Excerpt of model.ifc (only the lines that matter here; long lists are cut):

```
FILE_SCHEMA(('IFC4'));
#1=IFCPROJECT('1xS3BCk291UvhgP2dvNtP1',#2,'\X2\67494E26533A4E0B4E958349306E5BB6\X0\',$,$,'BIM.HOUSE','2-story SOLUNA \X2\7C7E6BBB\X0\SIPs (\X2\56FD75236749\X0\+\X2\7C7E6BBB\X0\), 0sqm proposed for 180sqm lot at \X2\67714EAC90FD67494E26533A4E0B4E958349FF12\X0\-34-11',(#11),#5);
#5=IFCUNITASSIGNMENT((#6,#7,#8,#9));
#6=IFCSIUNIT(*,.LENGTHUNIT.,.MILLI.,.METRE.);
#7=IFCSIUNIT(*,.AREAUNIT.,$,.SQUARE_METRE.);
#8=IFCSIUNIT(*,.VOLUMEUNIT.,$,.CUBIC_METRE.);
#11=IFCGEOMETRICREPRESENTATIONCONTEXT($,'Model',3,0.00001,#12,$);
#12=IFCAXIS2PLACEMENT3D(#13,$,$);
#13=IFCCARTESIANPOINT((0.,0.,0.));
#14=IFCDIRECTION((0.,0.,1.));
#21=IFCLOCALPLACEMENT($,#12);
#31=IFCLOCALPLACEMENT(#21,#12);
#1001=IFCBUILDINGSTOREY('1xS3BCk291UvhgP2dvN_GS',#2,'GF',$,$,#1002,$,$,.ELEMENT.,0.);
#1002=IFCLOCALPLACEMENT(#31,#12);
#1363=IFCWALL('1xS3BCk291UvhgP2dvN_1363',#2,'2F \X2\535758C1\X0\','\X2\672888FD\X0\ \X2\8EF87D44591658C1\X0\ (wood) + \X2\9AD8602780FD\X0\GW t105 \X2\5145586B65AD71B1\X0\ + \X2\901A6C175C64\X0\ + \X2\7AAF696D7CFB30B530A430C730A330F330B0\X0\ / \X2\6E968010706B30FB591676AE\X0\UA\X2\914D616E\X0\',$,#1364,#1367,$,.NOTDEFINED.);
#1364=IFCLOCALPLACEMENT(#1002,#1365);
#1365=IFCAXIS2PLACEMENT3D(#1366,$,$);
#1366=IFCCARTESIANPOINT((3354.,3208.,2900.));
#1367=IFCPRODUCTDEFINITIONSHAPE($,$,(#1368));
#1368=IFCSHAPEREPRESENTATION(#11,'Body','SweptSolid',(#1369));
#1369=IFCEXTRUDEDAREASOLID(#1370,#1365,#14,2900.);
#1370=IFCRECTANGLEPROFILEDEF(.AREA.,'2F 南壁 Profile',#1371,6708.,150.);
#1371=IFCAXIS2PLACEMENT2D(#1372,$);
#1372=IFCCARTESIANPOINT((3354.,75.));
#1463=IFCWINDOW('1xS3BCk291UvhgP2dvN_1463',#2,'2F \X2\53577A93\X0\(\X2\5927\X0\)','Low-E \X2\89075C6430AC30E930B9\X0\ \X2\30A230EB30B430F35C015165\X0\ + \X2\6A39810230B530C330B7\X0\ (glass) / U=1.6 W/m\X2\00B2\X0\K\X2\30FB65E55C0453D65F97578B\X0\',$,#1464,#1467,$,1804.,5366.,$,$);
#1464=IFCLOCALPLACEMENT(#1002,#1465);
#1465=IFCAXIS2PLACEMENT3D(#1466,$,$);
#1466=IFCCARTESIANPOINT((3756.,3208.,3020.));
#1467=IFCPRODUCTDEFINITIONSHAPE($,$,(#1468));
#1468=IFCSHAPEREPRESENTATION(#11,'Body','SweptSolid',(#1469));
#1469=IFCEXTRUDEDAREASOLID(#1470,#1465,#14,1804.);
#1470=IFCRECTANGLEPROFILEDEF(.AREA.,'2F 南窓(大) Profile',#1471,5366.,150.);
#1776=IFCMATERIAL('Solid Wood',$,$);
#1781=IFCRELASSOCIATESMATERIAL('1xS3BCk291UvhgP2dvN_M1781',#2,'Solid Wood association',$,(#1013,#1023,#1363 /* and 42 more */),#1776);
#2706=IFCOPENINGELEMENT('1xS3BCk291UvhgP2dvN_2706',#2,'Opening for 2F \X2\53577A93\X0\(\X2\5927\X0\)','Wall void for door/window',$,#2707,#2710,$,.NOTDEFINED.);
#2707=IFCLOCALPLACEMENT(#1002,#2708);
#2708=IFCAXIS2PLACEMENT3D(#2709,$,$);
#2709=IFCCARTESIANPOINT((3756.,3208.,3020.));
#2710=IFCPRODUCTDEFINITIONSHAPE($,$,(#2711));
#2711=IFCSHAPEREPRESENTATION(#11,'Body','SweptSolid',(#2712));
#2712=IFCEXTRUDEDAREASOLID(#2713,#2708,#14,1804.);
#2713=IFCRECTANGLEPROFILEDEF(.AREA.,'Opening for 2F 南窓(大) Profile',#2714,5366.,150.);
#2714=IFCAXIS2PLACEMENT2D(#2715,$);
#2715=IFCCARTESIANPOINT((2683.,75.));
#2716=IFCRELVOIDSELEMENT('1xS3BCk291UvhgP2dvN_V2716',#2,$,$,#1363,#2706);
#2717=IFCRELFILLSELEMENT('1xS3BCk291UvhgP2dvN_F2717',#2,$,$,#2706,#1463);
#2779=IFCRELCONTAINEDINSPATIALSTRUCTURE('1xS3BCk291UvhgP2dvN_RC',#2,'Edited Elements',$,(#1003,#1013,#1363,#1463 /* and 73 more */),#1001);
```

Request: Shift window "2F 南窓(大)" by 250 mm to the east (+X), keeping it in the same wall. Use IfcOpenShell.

```python
import ifcopenshell
import ifcopenshell.api.geometry
import ifcopenshell.util.placement
import ifcopenshell.util.unit

model = ifcopenshell.open("model.ifc")
unit_scale = ifcopenshell.util.unit.calculate_unit_scale(model)

window = model.by_guid("1xS3BCk291UvhgP2dvN_1463")
opening = window.FillsVoids[0].RelatingOpeningElement
wall = opening.VoidsElements[0].RelatingBuildingElement

wall_matrix = ifcopenshell.util.placement.get_local_placement(wall.ObjectPlacement)
shift = wall_matrix[:3, 0] * 0.25 / unit_scale
before = ifcopenshell.util.placement.get_local_placement(window.ObjectPlacement)[:3, 3].copy()

# The window is not placed relative to its opening, so move both.
for product in (opening, window):
    matrix = ifcopenshell.util.placement.get_local_placement(product.ObjectPlacement)
    matrix[:3, 3] += shift
    ifcopenshell.api.geometry.edit_object_placement(model, product=product, matrix=matrix, is_si=False)

after = ifcopenshell.util.placement.get_local_placement(window.ObjectPlacement)[:3, 3]
print("window moved by", (after - before).round(3) + 0.0)

model.write("model_updated.ifc")
```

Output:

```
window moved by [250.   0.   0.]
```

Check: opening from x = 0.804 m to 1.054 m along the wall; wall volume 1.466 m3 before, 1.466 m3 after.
